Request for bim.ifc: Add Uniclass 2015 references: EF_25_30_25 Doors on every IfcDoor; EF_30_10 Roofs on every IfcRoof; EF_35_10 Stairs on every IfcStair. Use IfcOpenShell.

First a look at what the model holds.

```python
import ifcopenshell

model = ifcopenshell.open("bim.ifc")
print(model.schema)
print("classifications:", [c.Name for c in model.by_type("IfcClassification")])
for ifc_class in ("IfcDoor", "IfcRoof", "IfcStair", "IfcWall", "IfcWindow"):
    print(ifc_class, len(model.by_type(ifc_class)))
```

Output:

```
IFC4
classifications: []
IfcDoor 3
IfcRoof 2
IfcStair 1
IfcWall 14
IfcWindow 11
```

```python
import ifcopenshell
import ifcopenshell.api.classification

model = ifcopenshell.open("bim.ifc")

system = ifcopenshell.api.classification.add_classification(model, classification="Uniclass 2015")

codes = {
    "IfcDoor": ("EF_25_30_25", "Doors"),
    "IfcRoof": ("EF_30_10", "Roofs"),
    "IfcStair": ("EF_35_10", "Stairs"),
}
for ifc_class, (code, name) in codes.items():
    products = model.by_type(ifc_class)
    ifcopenshell.api.classification.add_reference(
        model, products=products, classification=system, identification=code, name=name
    )
    print(code, len(products))

model.write("bim_edited.ifc")
```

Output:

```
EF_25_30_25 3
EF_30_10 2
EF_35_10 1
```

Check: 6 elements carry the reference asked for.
